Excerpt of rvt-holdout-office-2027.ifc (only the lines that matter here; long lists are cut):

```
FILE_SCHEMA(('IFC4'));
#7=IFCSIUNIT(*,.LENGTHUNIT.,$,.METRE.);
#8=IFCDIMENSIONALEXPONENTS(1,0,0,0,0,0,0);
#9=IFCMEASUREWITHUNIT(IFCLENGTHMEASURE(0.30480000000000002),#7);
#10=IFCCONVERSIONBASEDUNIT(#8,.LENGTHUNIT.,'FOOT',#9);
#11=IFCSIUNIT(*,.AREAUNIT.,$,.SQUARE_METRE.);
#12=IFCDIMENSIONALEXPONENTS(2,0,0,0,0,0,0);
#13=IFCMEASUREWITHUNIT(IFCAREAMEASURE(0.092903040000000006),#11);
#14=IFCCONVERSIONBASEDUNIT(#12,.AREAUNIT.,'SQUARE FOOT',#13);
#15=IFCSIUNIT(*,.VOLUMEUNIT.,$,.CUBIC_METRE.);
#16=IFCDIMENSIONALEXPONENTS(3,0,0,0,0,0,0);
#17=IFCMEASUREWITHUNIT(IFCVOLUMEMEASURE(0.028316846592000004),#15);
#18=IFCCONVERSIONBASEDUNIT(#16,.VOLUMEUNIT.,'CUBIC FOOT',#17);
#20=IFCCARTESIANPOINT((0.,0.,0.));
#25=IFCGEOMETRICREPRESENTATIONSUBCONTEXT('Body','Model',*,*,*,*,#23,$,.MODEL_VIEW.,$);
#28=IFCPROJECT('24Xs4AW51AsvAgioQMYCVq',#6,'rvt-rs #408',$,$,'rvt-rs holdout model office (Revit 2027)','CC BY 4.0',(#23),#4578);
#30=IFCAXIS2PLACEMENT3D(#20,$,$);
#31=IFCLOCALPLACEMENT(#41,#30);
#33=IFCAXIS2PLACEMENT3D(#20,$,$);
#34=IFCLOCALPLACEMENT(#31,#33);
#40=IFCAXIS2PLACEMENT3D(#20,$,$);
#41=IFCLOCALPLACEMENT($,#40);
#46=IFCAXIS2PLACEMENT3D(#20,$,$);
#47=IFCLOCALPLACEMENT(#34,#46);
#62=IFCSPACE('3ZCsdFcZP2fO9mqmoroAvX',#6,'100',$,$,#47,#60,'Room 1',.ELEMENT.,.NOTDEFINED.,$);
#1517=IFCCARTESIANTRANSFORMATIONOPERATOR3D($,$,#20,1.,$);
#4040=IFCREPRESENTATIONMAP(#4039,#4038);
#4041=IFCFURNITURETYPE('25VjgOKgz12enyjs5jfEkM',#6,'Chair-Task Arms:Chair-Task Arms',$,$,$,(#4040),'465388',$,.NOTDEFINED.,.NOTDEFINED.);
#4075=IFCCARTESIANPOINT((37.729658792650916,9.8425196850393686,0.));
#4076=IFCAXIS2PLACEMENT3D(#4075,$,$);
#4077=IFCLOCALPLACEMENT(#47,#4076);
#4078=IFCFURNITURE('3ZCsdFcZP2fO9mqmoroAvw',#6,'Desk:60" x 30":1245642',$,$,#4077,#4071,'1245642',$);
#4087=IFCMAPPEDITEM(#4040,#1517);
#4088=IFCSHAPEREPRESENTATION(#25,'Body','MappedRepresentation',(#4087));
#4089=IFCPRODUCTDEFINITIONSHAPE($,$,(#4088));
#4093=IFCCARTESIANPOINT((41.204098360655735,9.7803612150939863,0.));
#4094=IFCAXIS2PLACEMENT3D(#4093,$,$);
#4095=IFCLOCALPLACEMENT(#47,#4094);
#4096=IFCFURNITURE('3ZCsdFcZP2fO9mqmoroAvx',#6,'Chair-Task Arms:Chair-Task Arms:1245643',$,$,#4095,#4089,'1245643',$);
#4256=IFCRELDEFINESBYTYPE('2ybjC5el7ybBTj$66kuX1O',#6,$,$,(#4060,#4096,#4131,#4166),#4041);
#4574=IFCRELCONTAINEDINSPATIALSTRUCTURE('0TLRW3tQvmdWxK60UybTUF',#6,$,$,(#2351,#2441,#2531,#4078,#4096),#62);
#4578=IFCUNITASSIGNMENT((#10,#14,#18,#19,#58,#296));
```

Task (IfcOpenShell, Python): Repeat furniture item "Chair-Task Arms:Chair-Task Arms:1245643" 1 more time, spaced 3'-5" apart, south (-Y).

```python
import numpy as np
import ifcopenshell
import ifcopenshell.api.geometry
import ifcopenshell.api.root
import ifcopenshell.util.element
import ifcopenshell.util.placement
import ifcopenshell.util.unit

model = ifcopenshell.open("rvt-holdout-office-2027.ifc")
unit_scale = ifcopenshell.util.unit.calculate_unit_scale(model)


def reuse_history(source, copy):
    """copy_class also copies each property set's owner history, people and application; keep the originals."""
    for rel in copy.IsDefinedBy:
        if rel.is_a("IfcRelDefinesByProperties") and (history := rel.RelatingPropertyDefinition.OwnerHistory):
            rel.RelatingPropertyDefinition.OwnerHistory = source.OwnerHistory
            ifcopenshell.util.element.remove_deep2(model, history)


source = model.by_id(4096)
base = ifcopenshell.util.placement.get_local_placement(source.ObjectPlacement)
step = np.array([0.0, -1.0, 0.0]) * 41 * 0.0254 / unit_scale

for i in range(1, 2):
    copy = ifcopenshell.api.root.copy_class(model, product=source)
    copy.Representation = ifcopenshell.util.element.copy_deep(
        model, source.Representation, exclude=["IfcGeometricRepresentationContext", "IfcRepresentationMap"]
    )
    copy.Name = "Chair-Task Arms:Chair-Task Arms"
    copy.Tag = None
    reuse_history(source, copy)
    matrix = base.copy()
    matrix[:3, 3] += i * step
    print("added at", matrix[:3, 3].round(3) + 0.0)
    ifcopenshell.api.geometry.edit_object_placement(model, product=copy, matrix=matrix, is_si=False)

model.write("rvt-holdout-office-2027_updated.ifc")
```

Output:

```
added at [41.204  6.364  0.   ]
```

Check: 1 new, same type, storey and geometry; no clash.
